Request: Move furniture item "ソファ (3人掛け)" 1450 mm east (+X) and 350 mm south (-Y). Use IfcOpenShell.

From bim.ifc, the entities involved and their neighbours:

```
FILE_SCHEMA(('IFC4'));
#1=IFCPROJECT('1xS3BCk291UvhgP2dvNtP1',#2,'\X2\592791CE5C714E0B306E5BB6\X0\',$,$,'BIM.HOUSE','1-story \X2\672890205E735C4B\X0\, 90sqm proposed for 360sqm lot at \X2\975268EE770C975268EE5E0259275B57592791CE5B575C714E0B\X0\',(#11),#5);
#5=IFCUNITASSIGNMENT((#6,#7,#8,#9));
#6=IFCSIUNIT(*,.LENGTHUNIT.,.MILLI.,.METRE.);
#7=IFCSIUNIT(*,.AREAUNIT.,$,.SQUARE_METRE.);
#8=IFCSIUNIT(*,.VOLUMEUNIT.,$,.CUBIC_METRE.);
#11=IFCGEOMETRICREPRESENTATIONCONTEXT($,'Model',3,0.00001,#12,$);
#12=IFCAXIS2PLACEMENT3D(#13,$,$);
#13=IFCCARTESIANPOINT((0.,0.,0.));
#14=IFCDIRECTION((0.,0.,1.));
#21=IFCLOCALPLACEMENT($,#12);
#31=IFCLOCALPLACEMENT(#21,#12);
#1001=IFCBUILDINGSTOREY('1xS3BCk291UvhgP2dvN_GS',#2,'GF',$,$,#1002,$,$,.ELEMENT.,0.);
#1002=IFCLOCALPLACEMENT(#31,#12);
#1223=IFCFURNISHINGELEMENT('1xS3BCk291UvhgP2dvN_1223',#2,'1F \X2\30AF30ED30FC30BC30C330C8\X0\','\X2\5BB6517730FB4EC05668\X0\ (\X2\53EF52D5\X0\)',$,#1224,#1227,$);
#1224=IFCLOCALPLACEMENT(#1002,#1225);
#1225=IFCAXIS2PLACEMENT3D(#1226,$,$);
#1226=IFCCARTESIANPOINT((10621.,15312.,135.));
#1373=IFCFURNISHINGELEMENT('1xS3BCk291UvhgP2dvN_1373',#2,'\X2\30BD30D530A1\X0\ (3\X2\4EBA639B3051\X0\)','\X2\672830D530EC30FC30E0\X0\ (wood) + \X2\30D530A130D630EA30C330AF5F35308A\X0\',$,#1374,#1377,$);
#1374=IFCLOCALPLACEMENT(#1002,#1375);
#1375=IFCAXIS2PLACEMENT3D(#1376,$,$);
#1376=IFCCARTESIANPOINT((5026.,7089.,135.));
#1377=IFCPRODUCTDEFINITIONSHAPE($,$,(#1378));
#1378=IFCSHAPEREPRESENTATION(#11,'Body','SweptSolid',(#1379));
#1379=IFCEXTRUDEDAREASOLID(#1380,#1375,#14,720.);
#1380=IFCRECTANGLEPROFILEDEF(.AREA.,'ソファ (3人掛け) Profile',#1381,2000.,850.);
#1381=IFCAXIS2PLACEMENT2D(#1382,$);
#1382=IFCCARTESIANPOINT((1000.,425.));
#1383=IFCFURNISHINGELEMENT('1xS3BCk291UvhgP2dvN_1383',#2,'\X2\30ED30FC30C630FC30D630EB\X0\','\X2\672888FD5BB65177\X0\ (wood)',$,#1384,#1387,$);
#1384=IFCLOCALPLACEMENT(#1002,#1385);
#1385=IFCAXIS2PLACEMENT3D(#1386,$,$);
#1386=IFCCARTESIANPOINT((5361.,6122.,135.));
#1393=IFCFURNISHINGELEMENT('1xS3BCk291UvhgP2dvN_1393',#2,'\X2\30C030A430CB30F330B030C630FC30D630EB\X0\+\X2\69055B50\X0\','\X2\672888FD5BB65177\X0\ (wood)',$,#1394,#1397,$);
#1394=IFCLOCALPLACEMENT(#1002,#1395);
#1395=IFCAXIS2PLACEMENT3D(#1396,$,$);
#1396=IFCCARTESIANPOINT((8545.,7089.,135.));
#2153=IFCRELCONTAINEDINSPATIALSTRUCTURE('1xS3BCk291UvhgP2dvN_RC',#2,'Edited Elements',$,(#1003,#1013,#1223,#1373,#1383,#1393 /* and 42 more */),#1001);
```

```python
import ifcopenshell
import ifcopenshell.api.geometry
import ifcopenshell.util.placement
import ifcopenshell.util.unit

model = ifcopenshell.open("bim.ifc")
unit_scale = ifcopenshell.util.unit.calculate_unit_scale(model)

item = model.by_guid("1xS3BCk291UvhgP2dvN_1373")
matrix = ifcopenshell.util.placement.get_local_placement(item.ObjectPlacement)
matrix[0, 3] += 1.45 / unit_scale
matrix[1, 3] -= 0.35 / unit_scale
ifcopenshell.api.geometry.edit_object_placement(model, product=item, matrix=matrix, is_si=False)

print(ifcopenshell.util.placement.get_local_placement(item.ObjectPlacement).round(3) + 0.0)

model.write("bim_v2.ifc")
```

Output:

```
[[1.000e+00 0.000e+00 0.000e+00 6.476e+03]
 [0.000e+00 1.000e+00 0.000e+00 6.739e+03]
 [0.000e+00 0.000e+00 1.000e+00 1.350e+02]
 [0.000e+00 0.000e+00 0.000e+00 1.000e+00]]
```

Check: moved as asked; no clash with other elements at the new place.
